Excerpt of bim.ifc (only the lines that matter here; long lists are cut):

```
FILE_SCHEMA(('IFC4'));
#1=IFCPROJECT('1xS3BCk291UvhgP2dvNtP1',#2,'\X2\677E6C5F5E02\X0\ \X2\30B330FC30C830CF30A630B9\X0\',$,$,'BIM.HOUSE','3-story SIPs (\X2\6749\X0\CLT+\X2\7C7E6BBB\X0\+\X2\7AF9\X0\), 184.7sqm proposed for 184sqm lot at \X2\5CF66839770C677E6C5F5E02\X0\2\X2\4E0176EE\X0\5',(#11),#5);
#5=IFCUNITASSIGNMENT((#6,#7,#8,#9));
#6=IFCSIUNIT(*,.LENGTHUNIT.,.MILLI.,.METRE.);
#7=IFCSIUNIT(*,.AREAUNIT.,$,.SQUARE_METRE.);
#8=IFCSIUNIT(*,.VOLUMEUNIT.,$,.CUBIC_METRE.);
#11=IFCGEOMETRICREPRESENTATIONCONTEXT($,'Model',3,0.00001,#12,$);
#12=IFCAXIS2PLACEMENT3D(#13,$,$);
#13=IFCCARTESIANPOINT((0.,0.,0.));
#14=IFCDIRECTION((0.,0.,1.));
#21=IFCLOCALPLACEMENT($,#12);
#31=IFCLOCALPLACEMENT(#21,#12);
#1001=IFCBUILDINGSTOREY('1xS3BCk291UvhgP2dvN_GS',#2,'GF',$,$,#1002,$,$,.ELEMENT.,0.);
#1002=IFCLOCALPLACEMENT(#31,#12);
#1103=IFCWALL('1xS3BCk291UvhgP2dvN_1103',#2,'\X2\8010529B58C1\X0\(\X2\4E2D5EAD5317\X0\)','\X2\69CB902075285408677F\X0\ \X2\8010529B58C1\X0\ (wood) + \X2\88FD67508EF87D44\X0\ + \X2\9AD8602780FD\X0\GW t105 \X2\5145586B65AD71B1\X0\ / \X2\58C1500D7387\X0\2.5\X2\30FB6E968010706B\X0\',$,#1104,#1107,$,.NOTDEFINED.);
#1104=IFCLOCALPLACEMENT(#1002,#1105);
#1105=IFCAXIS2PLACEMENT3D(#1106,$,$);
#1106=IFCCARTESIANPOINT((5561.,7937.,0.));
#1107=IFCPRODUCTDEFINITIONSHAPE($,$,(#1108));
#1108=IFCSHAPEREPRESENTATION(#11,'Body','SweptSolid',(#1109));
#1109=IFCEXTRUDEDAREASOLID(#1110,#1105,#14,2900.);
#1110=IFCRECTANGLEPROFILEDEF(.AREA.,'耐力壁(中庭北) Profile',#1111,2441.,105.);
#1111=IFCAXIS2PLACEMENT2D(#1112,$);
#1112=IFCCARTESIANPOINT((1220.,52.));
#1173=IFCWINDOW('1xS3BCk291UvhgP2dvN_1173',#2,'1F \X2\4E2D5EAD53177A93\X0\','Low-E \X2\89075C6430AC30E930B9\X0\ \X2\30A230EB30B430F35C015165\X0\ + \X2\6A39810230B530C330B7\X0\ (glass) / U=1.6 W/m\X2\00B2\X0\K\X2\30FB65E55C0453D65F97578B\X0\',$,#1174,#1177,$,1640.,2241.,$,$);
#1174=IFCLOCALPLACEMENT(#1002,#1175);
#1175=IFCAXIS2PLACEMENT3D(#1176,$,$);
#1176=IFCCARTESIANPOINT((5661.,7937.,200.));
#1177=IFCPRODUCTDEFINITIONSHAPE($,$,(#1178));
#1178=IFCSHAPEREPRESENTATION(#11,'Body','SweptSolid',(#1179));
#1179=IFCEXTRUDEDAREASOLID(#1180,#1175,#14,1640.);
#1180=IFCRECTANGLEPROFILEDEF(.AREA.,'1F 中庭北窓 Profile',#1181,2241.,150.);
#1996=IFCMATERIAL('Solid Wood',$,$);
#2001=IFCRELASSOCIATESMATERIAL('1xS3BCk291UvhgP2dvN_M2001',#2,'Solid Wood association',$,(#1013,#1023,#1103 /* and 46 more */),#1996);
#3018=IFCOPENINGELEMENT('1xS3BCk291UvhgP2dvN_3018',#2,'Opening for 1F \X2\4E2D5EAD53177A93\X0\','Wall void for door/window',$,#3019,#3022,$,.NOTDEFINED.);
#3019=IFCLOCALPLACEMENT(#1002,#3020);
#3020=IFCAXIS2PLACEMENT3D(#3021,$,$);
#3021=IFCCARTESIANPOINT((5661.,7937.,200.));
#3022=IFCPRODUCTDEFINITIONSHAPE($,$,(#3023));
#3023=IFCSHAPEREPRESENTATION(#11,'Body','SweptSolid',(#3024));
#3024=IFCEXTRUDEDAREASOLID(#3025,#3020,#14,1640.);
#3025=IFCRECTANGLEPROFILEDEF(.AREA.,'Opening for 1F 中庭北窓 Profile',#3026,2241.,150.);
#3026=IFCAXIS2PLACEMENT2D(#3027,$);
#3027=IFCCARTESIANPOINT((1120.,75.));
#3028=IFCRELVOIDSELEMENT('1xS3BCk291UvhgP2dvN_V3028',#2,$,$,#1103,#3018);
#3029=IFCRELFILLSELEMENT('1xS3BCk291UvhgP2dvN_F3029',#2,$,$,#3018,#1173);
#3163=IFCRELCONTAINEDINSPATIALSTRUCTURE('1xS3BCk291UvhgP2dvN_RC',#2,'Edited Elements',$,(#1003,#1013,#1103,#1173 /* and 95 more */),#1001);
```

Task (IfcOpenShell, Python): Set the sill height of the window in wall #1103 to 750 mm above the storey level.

```python
import numpy as np
import ifcopenshell
import ifcopenshell.api.geometry
import ifcopenshell.geom
import ifcopenshell.util.element
import ifcopenshell.util.placement
import ifcopenshell.util.shape
import ifcopenshell.util.unit

model = ifcopenshell.open("bim.ifc")
unit_scale = ifcopenshell.util.unit.calculate_unit_scale(model)

window = model.by_id(1173)
opening = window.FillsVoids[0].RelatingOpeningElement
storey = ifcopenshell.util.element.get_container(window, ifc_class="IfcBuildingStorey")
level = ifcopenshell.util.placement.get_local_placement(storey.ObjectPlacement)[2, 3]

# The opening's origin need not be at the sill, so measure its lowest point.
shape = ifcopenshell.geom.create_shape(ifcopenshell.geom.settings(), opening)
bottom = ifcopenshell.util.shape.get_shape_bottom_elevation(shape, shape.geometry) / unit_scale
dz = level + 750.0 - bottom

shift = np.array([0.0, 0.0, dz])
# The window is not placed relative to its opening, so move both.
for product in (opening, window):
    matrix = ifcopenshell.util.placement.get_local_placement(product.ObjectPlacement)
    matrix[:3, 3] += shift
    ifcopenshell.api.geometry.edit_object_placement(model, product=product, matrix=matrix, is_si=False)

print(f"moved by {dz * unit_scale:+.3f} m")

model.write("bim_edited.ifc")
```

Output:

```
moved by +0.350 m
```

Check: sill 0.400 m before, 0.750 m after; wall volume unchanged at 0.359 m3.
